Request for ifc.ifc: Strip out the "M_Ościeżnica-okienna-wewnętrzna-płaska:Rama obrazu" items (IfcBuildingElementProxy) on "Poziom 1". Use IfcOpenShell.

First a look at what the model holds.

```python
import ifcopenshell
import ifcopenshell.util.element

model = ifcopenshell.open("ifc.ifc")
print(model.schema)
storey = next(s for s in model.by_type("IfcBuildingStorey") if s.Name == "Poziom 1")
proxies = [e for e in ifcopenshell.util.element.get_decomposition(storey) if e.is_a("IfcBuildingElementProxy")]
seen = {}
for e in proxies:
    element_type = ifcopenshell.util.element.get_type(e)
    name = element_type.Name if element_type not in (None, e) else None
    seen[name] = seen.get(name, 0) + 1
for name, count in sorted(seen.items(), key=str):
    print(count, "x", name)
```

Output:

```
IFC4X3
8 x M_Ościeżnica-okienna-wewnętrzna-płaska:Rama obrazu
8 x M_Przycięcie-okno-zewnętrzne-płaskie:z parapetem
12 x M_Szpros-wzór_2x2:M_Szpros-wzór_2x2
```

```python
import ifcopenshell
import ifcopenshell.api.root
import ifcopenshell.util.element

model = ifcopenshell.open("ifc.ifc")

storey = next(s for s in model.by_type("IfcBuildingStorey") if s.Name == "Poziom 1")
proxies = [e for e in ifcopenshell.util.element.get_decomposition(storey) if e.is_a("IfcBuildingElementProxy")]
targets = [e for e in proxies if (t := ifcopenshell.util.element.get_type(e)) not in (None, e) and t.Name == "M_Ościeżnica-okienna-wewnętrzna-płaska:Rama obrazu"]

for e in targets:
    ifcopenshell.api.root.remove_product(model, product=e)
print(len(targets), "removed")

model.write("ifc_edited.ifc")
```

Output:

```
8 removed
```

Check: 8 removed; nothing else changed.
